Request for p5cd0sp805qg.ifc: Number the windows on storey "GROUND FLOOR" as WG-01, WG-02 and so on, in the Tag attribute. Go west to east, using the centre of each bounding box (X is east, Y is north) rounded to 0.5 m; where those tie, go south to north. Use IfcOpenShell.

First a look at what the model holds.

```python
import ifcopenshell
import ifcopenshell.util.element
import ifcopenshell.util.placement

model = ifcopenshell.open("p5cd0sp805qg.ifc")
print(model.schema)
storey = next(s for s in model.by_type("IfcBuildingStorey") if s.Name == "GROUND FLOOR")
windows = [e for e in ifcopenshell.util.element.get_decomposition(storey) if e.is_a("IfcWindow")]
for e in sorted(windows, key=lambda e: e.id()):
    origin = ifcopenshell.util.placement.get_local_placement(e.ObjectPlacement)[:3, 3]
    print(e.id(), e.Tag, e.Name, origin.round(2) + 0.0, sep=" | ")
```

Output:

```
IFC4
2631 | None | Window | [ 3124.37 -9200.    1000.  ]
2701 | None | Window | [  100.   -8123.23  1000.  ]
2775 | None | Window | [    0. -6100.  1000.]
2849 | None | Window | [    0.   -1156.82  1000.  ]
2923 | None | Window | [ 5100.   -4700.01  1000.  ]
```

```python
import ifcopenshell
import ifcopenshell.geom
import ifcopenshell.util.element
import ifcopenshell.util.shape

model = ifcopenshell.open("p5cd0sp805qg.ifc")
settings = ifcopenshell.geom.settings()
settings.set("use-world-coords", True)


def centre(element):
    shape = ifcopenshell.geom.create_shape(settings, element)
    return ifcopenshell.util.shape.get_bbox_centroid(shape.geometry)


storey = next(s for s in model.by_type("IfcBuildingStorey") if s.Name == "GROUND FLOOR")
windows = [e for e in ifcopenshell.util.element.get_decomposition(storey) if e.is_a("IfcWindow")]

# Insertion points can sit at a corner or the storey origin, so sort by the geometry (in metres).
centres = {e: centre(e) for e in windows}
windows.sort(key=lambda e: (round(centres[e][0] / 0.5), centres[e][1]))

for i, e in enumerate(windows, start=1):
    number = f"WG-{i:02d}"
    e.Tag = number
    print(e.id(), number)

model.write("p5cd0sp805qg-out.ifc")
```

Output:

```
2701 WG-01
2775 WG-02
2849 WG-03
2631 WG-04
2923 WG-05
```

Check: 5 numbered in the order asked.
